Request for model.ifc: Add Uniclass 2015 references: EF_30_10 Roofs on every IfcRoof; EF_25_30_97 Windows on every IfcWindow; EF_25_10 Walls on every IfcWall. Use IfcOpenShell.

First a look at what the model holds.

```python
import ifcopenshell

model = ifcopenshell.open("model.ifc")
print(model.schema)
print("classifications:", [c.Name for c in model.by_type("IfcClassification")])
for ifc_class in ("IfcDoor", "IfcRoof", "IfcStair", "IfcWall", "IfcWindow"):
    print(ifc_class, len(model.by_type(ifc_class)))
```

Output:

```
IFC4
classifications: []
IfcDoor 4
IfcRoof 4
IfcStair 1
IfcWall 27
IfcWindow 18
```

```python
import ifcopenshell
import ifcopenshell.api.classification

model = ifcopenshell.open("model.ifc")

system = ifcopenshell.api.classification.add_classification(model, classification="Uniclass 2015")

codes = {
    "IfcRoof": ("EF_30_10", "Roofs"),
    "IfcWindow": ("EF_25_30_97", "Windows"),
    "IfcWall": ("EF_25_10", "Walls"),
}
for ifc_class, (code, name) in codes.items():
    products = model.by_type(ifc_class)
    ifcopenshell.api.classification.add_reference(
        model, products=products, classification=system, identification=code, name=name
    )
    print(code, len(products))

model.write("model_updated.ifc")
```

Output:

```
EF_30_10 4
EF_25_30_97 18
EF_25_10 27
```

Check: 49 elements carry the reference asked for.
